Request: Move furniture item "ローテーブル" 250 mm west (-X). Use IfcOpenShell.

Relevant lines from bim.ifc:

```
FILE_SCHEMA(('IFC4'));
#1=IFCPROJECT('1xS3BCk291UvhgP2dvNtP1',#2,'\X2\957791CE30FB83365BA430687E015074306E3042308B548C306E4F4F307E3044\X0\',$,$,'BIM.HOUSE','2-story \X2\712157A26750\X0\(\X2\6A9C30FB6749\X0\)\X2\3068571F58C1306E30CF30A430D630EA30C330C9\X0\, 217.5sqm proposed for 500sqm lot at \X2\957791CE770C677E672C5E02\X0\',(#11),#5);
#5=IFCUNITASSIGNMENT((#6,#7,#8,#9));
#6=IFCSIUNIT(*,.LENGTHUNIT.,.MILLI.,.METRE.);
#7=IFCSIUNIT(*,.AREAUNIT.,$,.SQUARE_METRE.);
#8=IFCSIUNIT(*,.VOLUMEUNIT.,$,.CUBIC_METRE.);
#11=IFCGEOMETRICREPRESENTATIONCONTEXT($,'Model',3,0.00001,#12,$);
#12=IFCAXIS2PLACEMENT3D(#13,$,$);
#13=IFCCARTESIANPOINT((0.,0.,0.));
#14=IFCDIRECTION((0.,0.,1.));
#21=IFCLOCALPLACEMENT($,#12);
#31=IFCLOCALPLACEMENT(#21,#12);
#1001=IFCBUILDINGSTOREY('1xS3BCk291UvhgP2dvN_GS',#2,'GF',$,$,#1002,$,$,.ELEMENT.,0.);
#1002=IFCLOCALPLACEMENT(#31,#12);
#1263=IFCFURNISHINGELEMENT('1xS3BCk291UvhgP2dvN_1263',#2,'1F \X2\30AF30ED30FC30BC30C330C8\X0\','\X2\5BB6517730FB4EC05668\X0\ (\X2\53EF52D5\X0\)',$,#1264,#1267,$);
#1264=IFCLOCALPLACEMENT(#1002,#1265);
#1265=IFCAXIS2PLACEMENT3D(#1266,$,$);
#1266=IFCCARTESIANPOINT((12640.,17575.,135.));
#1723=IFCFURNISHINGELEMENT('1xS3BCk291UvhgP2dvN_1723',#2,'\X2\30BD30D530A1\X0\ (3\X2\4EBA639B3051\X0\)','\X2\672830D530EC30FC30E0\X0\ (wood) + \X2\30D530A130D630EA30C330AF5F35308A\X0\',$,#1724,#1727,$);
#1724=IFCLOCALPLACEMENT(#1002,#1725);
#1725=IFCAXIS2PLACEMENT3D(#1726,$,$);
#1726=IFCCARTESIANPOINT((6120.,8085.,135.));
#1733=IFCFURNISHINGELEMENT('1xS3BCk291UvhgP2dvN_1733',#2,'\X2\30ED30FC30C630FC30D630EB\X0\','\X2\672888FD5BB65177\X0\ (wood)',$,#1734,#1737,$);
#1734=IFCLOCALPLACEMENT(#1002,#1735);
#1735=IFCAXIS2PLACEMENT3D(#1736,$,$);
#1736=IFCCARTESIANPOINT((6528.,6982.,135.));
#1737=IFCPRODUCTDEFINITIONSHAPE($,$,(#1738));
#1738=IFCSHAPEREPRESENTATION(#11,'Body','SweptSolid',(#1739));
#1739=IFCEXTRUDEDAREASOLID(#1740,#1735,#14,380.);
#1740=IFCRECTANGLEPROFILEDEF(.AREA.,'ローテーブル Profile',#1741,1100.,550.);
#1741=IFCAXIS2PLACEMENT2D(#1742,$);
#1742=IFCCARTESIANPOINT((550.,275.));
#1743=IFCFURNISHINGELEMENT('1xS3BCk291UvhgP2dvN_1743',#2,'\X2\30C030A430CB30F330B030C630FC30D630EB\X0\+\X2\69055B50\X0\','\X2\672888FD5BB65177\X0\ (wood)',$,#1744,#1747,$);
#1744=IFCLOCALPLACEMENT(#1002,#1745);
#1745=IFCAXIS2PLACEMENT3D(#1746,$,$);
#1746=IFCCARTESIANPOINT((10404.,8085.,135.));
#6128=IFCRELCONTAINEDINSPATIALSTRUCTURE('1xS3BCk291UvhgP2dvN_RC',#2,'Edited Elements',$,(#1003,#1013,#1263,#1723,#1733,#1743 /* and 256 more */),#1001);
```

```python
import ifcopenshell
import ifcopenshell.api.geometry
import ifcopenshell.util.placement
import ifcopenshell.util.unit

model = ifcopenshell.open("bim.ifc")
unit_scale = ifcopenshell.util.unit.calculate_unit_scale(model)

item = model.by_id(1733)
matrix = ifcopenshell.util.placement.get_local_placement(item.ObjectPlacement)
matrix[0, 3] -= 0.25 / unit_scale
ifcopenshell.api.geometry.edit_object_placement(model, product=item, matrix=matrix, is_si=False)

print(ifcopenshell.util.placement.get_local_placement(item.ObjectPlacement).round(3) + 0.0)

model.write("bim_rev.ifc")
```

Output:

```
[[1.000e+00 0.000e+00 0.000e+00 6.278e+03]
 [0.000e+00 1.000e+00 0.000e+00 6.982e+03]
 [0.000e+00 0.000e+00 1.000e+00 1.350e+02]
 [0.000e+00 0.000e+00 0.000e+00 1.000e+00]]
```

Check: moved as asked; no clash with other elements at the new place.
